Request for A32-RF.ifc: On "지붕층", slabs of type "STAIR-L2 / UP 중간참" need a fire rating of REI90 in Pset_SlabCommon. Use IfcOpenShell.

First a look at what the model holds.

```python
import ifcopenshell
import ifcopenshell.util.element

model = ifcopenshell.open("A32-RF.ifc")
print(model.schema)
storey = next(s for s in model.by_type("IfcBuildingStorey") if s.Name == "지붕층")
slabs = [e for e in ifcopenshell.util.element.get_decomposition(storey) if e.is_a("IfcSlab")]
seen = {}
for e in slabs:
    element_type = ifcopenshell.util.element.get_type(e)
    key = (element_type.Name if element_type != e and element_type else None, ifcopenshell.util.element.get_pset(e, "Pset_SlabCommon", "FireRating"))
    seen[key] = seen.get(key, 0) + 1
for (name, value), count in sorted(seen.items(), key=str):
    print(count, "x", name, "|", value)
```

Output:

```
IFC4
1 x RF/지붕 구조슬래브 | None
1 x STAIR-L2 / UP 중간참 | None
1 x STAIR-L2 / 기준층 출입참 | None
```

```python
import ifcopenshell
import ifcopenshell.api.pset
import ifcopenshell.util.element

model = ifcopenshell.open("A32-RF.ifc")

storey = next(s for s in model.by_type("IfcBuildingStorey") if s.Name == "지붕층")
slabs = [e for e in ifcopenshell.util.element.get_decomposition(storey) if e.is_a("IfcSlab")]

count = 0
for e in slabs:
    element_type = ifcopenshell.util.element.get_type(e)
    if element_type in (None, e) or element_type.Name != "STAIR-L2 / UP 중간참":
        continue
    # add_pset returns the element's existing set when there is one.
    pset = ifcopenshell.api.pset.add_pset(model, product=e, name="Pset_SlabCommon")
    ifcopenshell.api.pset.edit_pset(model, pset=pset, properties={"FireRating": "REI90"})
    count += 1

print(count, "slabs updated")

model.write("A32-RF_rev.ifc")
```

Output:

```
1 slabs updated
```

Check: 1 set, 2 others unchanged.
